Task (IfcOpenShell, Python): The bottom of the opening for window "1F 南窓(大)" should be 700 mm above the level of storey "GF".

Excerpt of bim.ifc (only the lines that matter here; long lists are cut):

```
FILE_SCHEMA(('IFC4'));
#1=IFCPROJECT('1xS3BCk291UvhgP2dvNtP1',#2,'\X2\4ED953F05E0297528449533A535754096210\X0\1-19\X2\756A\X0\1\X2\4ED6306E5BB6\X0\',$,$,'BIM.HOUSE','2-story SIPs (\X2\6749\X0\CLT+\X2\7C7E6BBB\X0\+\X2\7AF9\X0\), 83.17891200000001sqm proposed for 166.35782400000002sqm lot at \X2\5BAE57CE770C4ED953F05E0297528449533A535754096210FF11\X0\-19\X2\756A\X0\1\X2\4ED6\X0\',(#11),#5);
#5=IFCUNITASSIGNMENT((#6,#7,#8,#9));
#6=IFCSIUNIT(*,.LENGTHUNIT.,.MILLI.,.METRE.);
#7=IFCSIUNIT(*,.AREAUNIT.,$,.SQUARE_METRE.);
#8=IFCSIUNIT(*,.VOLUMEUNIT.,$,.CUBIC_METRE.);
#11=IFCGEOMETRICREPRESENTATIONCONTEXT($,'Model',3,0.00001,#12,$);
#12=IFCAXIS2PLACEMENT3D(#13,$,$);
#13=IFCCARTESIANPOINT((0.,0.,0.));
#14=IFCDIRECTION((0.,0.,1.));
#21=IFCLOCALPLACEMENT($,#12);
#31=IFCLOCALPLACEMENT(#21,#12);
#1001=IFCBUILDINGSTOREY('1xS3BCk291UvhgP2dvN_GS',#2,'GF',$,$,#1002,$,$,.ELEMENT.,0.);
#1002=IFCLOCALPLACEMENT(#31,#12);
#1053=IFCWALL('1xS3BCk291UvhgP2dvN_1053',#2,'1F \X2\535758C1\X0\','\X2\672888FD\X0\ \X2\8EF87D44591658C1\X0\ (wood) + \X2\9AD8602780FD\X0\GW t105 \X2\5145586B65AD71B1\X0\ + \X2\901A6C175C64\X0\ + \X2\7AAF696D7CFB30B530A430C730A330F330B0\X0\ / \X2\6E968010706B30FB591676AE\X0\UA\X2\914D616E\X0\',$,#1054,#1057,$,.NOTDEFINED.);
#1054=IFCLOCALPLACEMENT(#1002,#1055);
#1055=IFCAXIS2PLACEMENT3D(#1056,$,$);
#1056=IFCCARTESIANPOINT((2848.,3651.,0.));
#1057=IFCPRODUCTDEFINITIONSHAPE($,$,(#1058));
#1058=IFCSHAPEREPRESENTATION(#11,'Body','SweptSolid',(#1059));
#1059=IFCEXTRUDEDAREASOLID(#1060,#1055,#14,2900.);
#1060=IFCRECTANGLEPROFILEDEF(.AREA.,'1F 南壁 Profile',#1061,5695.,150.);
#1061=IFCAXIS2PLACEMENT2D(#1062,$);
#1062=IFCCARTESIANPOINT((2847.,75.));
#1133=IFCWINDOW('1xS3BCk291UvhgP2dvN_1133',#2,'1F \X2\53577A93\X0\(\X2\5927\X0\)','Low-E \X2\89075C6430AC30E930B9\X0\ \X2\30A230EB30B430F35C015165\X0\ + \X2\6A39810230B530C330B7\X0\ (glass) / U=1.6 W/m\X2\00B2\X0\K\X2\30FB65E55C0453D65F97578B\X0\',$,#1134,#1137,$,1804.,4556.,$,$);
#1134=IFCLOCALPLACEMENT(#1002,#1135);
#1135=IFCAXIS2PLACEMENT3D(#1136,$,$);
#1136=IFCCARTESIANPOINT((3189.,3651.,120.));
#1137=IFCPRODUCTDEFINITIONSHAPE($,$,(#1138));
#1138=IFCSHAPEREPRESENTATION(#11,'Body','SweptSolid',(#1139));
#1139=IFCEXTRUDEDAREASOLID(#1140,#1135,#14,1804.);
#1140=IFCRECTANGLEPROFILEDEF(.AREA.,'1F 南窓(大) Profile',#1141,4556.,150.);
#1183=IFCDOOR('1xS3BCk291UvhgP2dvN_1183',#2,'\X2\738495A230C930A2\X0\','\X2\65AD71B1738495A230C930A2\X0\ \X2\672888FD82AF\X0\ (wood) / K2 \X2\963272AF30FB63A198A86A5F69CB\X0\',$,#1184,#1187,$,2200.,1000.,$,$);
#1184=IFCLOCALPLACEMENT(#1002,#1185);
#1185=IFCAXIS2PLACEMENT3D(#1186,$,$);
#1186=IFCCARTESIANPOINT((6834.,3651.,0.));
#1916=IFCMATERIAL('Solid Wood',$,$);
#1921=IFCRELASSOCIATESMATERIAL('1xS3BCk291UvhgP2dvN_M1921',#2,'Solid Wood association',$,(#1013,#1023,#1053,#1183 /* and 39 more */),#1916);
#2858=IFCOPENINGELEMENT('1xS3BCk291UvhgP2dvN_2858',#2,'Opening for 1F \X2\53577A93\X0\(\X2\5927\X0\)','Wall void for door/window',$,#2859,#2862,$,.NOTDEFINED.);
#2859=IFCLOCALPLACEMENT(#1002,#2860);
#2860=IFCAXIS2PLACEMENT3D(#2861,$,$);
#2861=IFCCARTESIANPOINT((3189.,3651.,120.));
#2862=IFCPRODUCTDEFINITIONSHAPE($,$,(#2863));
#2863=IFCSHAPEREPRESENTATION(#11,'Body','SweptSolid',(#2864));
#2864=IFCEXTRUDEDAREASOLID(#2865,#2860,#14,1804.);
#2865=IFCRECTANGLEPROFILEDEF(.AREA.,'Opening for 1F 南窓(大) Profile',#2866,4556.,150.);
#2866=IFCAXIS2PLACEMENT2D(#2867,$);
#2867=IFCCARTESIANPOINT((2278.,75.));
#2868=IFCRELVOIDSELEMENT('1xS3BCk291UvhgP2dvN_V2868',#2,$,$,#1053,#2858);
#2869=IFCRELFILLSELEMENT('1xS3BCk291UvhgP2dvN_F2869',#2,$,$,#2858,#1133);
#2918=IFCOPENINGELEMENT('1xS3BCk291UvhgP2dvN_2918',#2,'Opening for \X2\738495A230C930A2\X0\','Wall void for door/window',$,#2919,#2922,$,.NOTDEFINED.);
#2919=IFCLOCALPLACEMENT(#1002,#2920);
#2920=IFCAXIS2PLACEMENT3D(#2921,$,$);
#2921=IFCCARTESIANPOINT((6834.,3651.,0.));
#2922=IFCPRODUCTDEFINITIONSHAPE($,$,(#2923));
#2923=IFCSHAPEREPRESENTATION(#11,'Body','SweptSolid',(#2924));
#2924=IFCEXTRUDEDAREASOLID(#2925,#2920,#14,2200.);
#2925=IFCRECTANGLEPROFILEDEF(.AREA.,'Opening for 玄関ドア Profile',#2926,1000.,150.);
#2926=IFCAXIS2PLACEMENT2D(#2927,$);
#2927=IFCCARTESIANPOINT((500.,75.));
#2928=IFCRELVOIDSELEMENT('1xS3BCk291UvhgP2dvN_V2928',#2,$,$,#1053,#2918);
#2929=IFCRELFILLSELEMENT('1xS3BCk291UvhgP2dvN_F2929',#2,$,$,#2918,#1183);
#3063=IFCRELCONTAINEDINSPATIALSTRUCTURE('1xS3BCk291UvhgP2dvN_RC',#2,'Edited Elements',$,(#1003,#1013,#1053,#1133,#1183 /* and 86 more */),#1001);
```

```python
import numpy as np
import ifcopenshell
import ifcopenshell.api.geometry
import ifcopenshell.geom
import ifcopenshell.util.element
import ifcopenshell.util.placement
import ifcopenshell.util.shape
import ifcopenshell.util.unit

model = ifcopenshell.open("bim.ifc")
unit_scale = ifcopenshell.util.unit.calculate_unit_scale(model)

window = model.by_guid("1xS3BCk291UvhgP2dvN_1133")
opening = window.FillsVoids[0].RelatingOpeningElement
storey = ifcopenshell.util.element.get_container(window, ifc_class="IfcBuildingStorey")
level = ifcopenshell.util.placement.get_local_placement(storey.ObjectPlacement)[2, 3]

# The opening's origin need not be at the sill, so measure its lowest point.
shape = ifcopenshell.geom.create_shape(ifcopenshell.geom.settings(), opening)
bottom = ifcopenshell.util.shape.get_shape_bottom_elevation(shape, shape.geometry) / unit_scale
dz = level + 0.7 / unit_scale - bottom

shift = np.array([0.0, 0.0, dz])
# The window is not placed relative to its opening, so move both.
for product in (opening, window):
    matrix = ifcopenshell.util.placement.get_local_placement(product.ObjectPlacement)
    matrix[:3, 3] += shift
    ifcopenshell.api.geometry.edit_object_placement(model, product=product, matrix=matrix, is_si=False)

print(f"moved by {dz * unit_scale:+.3f} m")

model.write("bim_updated.ifc")
```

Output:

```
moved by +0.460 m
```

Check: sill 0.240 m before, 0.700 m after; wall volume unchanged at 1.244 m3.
